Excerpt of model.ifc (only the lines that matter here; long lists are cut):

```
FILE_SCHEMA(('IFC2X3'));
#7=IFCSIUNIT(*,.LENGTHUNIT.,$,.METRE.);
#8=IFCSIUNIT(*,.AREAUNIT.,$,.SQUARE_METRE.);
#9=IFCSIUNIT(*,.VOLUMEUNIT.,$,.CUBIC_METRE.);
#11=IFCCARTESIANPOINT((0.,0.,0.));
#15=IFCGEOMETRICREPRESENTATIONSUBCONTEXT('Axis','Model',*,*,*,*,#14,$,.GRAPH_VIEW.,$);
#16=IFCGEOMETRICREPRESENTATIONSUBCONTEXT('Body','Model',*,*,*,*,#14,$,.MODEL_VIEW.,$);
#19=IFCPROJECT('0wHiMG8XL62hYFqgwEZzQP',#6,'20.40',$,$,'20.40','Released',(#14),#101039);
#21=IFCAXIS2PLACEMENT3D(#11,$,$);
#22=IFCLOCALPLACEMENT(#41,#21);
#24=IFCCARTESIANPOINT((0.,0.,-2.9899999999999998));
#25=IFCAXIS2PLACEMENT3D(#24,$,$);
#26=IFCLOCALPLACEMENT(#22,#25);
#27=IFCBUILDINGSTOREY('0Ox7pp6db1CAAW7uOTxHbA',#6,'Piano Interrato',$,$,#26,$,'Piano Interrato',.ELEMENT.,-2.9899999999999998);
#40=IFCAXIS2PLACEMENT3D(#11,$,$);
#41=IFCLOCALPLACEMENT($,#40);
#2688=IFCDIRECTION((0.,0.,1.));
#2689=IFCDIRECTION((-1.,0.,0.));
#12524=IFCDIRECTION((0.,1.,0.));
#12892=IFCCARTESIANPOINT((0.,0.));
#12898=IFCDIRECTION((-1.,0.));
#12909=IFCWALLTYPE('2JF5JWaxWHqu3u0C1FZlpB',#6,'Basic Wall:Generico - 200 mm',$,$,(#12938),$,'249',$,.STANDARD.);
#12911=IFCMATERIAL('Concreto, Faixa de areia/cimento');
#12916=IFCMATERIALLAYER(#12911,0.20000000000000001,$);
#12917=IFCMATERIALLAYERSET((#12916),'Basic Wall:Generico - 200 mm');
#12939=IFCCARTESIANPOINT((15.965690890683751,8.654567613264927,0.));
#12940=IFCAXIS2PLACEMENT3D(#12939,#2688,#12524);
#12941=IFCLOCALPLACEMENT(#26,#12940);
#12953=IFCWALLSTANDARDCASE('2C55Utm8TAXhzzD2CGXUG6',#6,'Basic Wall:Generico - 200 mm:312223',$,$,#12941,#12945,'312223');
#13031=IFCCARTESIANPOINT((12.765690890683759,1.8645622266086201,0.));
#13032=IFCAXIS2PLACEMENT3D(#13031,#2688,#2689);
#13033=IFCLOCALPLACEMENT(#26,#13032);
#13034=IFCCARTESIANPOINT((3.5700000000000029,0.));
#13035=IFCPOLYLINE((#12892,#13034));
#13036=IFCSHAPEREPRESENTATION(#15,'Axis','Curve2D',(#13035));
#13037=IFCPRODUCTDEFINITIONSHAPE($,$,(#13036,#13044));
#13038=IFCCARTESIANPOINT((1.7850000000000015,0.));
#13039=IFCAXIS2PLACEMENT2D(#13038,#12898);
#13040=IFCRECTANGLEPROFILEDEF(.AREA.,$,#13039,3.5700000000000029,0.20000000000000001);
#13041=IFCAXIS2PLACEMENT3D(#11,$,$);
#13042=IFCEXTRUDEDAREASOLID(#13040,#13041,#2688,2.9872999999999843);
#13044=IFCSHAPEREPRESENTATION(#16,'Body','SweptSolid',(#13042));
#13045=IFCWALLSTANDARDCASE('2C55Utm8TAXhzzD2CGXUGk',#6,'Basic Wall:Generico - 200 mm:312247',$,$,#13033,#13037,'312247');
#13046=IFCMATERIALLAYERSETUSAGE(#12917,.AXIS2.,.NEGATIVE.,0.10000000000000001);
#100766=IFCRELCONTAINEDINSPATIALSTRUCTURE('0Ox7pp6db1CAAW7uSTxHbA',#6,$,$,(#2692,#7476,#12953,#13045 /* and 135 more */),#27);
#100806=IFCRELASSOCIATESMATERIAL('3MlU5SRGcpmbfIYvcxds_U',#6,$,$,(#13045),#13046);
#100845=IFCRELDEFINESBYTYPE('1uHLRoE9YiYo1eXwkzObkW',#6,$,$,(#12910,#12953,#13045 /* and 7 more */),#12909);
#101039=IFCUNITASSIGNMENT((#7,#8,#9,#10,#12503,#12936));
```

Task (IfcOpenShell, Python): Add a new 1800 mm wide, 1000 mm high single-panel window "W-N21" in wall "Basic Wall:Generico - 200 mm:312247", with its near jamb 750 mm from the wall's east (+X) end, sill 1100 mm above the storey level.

```python
import numpy as np
import ifcopenshell
import ifcopenshell.api.feature
import ifcopenshell.api.geometry
import ifcopenshell.api.root
import ifcopenshell.api.spatial
import ifcopenshell.api.type
import ifcopenshell.geom
import ifcopenshell.util.element
import ifcopenshell.util.placement
import ifcopenshell.util.representation
import ifcopenshell.util.shape
import ifcopenshell.util.unit

model = ifcopenshell.open("model.ifc")
unit_scale = ifcopenshell.util.unit.calculate_unit_scale(model)
settings = ifcopenshell.geom.settings()


def volume(element):
    """Net volume in cubic metres, openings subtracted."""
    shape = ifcopenshell.geom.create_shape(settings, element)
    return ifcopenshell.util.shape.get_volume(shape.geometry)


wall = model.by_guid("2C55Utm8TAXhzzD2CGXUGk")
storey = ifcopenshell.util.element.get_container(wall, ifc_class="IfcBuildingStorey")
context = ifcopenshell.util.representation.get_context(model, "Model", "Body", "MODEL_VIEW")
before = volume(wall)

width, height, from_end, sill = 1.8, 1, 0.75, 1.1  # metres

# The wall runs along its own X axis, and the end named is its -X end.
wall_shape = ifcopenshell.geom.create_shape(settings, wall)
x, y, z = ifcopenshell.util.shape.get_vertices(wall_shape.geometry).T
start = x.min() + from_end
face, thickness = float(y.min()), float(y.max() - y.min())
wall_matrix = ifcopenshell.util.placement.get_local_placement(wall.ObjectPlacement)
level = ifcopenshell.util.placement.get_local_placement(storey.ObjectPlacement)[2, 3]


def in_wall(x, y):
    """Placement at x, y metres in the wall's axes, at sill height."""
    matrix = wall_matrix.copy()
    matrix[:, 3] = wall_matrix @ np.array([x / unit_scale, y / unit_scale, 0.0, 1.0])
    matrix[2, 3] = level + sill / unit_scale
    return matrix


# Opening: a box that overshoots both wall faces by 50 mm.
opening = ifcopenshell.api.root.create_entity(model, ifc_class="IfcOpeningElement")
box = ifcopenshell.api.geometry.add_wall_representation(
    model, context=context, length=width, height=height, thickness=thickness + 0.1
)
ifcopenshell.api.geometry.assign_representation(model, product=opening, representation=box)
ifcopenshell.api.geometry.edit_object_placement(model, product=opening, matrix=in_wall(start, face - 0.05), is_si=False)
ifcopenshell.api.feature.add_feature(model, feature=opening, element=wall)

window = ifcopenshell.api.root.create_entity(model, ifc_class="IfcWindow", name="W-N21")
window.OverallWidth, window.OverallHeight = width / unit_scale, height / unit_scale
body = ifcopenshell.api.geometry.add_window_representation(
    model,
    context=context,
    overall_width=window.OverallWidth,
    overall_height=window.OverallHeight,
    partition_type="SINGLE_PANEL",
)
ifcopenshell.api.geometry.assign_representation(model, product=window, representation=body)
ifcopenshell.api.spatial.assign_container(model, products=[window], relating_structure=storey)
fills = ifcopenshell.api.feature.add_filling(model, opening=opening, element=window)
fills.OwnerHistory = window.OwnerHistory  # required in IFC2X3

# IFC2X3 keeps the operation on the window style.
style = ifcopenshell.api.root.create_entity(model, ifc_class="IfcWindowStyle", name="W-N21")
style.OperationType, style.ConstructionType = "SINGLE_PANEL", "NOTDEFINED"
style.ParameterTakesPrecedence = style.Sizeable = False
ifcopenshell.api.type.assign_type(model, related_objects=[window], relating_type=style)

# Centre the window in the wall's thickness.
ifcopenshell.api.geometry.edit_object_placement(model, product=window, matrix=in_wall(start, face), is_si=False)
window_shape = ifcopenshell.geom.create_shape(settings, window)
depth = ifcopenshell.util.shape.get_vertices(window_shape.geometry)[:, 1]
offset = face + thickness / 2 - (depth.min() + depth.max()) / 2
ifcopenshell.api.geometry.edit_object_placement(model, product=window, matrix=in_wall(start, offset), is_si=False)

after = volume(wall)

print(f"wall volume {before:.3f} -> {after:.3f} m3")

model.write("model_rev.ifc")
```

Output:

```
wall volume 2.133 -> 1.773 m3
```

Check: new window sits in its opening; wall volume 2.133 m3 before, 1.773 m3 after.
